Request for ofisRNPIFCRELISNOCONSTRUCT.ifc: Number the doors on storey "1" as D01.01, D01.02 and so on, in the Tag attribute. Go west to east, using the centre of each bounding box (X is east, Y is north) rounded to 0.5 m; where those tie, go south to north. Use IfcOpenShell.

First a look at what the model holds.

```python
import ifcopenshell
import ifcopenshell.util.element
import ifcopenshell.util.placement

model = ifcopenshell.open("ofisRNPIFCRELISNOCONSTRUCT.ifc")
print(model.schema)
storey = next(s for s in model.by_type("IfcBuildingStorey") if s.Name == "1")
doors = [e for e in ifcopenshell.util.element.get_decomposition(storey) if e.is_a("IfcDoor")]
for e in sorted(doors, key=lambda e: e.id()):
    origin = ifcopenshell.util.placement.get_local_placement(e.ObjectPlacement)[:3, 3]
    print(e.id(), e.Tag, e.Name, origin.round(2) + 0.0, sep=" | ")
```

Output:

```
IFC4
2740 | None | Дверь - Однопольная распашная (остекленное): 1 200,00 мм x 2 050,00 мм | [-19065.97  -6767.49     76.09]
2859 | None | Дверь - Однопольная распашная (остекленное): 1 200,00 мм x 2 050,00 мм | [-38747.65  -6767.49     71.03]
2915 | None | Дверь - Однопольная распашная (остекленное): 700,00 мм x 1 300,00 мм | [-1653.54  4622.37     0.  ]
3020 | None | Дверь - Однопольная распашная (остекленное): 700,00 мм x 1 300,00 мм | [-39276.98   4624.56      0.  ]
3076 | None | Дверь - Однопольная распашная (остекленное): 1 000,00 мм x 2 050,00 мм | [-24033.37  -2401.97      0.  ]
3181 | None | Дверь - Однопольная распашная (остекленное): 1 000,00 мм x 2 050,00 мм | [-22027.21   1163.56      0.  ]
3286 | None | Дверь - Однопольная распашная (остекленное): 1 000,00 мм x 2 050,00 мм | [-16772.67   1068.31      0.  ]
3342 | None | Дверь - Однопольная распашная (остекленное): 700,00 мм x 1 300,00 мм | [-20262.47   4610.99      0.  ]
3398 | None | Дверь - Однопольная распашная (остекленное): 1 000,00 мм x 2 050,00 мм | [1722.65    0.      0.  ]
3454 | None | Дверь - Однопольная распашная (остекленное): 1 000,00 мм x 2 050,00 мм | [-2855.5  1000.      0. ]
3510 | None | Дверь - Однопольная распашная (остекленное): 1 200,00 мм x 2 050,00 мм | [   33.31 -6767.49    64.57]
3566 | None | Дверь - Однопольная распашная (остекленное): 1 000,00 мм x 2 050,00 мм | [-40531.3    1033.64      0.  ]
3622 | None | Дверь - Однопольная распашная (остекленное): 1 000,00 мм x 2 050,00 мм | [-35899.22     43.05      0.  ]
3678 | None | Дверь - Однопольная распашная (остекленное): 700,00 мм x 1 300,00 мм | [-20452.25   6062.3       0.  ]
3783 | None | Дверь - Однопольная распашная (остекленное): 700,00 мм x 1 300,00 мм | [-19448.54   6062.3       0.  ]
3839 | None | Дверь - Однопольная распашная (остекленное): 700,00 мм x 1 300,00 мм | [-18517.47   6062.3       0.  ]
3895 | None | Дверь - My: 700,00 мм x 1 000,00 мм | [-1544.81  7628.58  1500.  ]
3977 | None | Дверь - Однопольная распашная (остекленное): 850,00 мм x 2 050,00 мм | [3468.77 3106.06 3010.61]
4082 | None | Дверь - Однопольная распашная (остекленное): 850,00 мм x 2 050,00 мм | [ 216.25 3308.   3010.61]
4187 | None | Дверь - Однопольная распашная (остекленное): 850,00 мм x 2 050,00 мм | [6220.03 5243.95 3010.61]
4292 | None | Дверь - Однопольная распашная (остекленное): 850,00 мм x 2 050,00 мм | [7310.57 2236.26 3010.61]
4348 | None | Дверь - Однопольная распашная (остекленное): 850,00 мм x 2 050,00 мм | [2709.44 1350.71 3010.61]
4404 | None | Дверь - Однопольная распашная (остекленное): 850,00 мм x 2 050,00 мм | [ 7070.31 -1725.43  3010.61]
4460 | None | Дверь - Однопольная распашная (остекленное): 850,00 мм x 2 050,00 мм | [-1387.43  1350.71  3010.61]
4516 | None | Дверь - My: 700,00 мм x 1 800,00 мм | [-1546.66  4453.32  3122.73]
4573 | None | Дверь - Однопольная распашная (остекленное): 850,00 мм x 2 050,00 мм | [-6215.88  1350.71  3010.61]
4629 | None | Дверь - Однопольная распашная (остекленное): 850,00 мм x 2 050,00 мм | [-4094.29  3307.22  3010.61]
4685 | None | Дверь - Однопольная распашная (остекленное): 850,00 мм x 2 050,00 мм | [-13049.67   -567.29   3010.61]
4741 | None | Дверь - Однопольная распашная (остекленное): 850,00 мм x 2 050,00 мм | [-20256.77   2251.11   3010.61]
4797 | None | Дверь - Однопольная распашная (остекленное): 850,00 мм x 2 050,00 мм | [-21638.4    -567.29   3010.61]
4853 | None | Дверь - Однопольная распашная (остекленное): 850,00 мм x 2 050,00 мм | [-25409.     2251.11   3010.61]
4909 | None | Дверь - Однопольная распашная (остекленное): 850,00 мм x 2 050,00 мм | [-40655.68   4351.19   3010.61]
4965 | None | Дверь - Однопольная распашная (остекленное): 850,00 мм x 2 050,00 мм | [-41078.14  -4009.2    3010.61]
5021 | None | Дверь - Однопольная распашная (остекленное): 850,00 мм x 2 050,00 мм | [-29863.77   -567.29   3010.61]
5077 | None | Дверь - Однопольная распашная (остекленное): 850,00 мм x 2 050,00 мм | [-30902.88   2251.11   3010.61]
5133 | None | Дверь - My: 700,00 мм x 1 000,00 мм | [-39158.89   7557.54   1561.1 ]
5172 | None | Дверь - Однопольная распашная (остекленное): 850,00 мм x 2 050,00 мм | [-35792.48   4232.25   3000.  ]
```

```python
import ifcopenshell
import ifcopenshell.geom
import ifcopenshell.util.element
import ifcopenshell.util.shape

model = ifcopenshell.open("ofisRNPIFCRELISNOCONSTRUCT.ifc")
settings = ifcopenshell.geom.settings()
settings.set("use-world-coords", True)


def centre(element):
    shape = ifcopenshell.geom.create_shape(settings, element)
    return ifcopenshell.util.shape.get_bbox_centroid(shape.geometry)


storey = next(s for s in model.by_type("IfcBuildingStorey") if s.Name == "1")
doors = [e for e in ifcopenshell.util.element.get_decomposition(storey) if e.is_a("IfcDoor")]

# Insertion points can sit at a corner or the storey origin, so sort by the geometry (in metres).
centres = {e: centre(e) for e in doors}
doors.sort(key=lambda e: (round(centres[e][0] / 0.5), centres[e][1]))

for i, e in enumerate(doors, start=1):
    number = f"D01.{i:02d}"
    e.Tag = number
    print(e.id(), number)

model.write("ofisRNPIFCRELISNOCONSTRUCT_rev.ifc")
```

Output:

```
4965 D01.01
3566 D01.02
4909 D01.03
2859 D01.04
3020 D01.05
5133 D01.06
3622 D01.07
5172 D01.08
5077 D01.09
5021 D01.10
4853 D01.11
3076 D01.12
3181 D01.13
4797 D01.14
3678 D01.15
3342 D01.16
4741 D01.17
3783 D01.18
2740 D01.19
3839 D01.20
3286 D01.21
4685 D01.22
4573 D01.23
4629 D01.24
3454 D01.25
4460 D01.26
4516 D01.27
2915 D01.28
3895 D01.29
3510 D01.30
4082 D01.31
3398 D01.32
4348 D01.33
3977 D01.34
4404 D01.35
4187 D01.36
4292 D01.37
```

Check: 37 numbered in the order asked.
